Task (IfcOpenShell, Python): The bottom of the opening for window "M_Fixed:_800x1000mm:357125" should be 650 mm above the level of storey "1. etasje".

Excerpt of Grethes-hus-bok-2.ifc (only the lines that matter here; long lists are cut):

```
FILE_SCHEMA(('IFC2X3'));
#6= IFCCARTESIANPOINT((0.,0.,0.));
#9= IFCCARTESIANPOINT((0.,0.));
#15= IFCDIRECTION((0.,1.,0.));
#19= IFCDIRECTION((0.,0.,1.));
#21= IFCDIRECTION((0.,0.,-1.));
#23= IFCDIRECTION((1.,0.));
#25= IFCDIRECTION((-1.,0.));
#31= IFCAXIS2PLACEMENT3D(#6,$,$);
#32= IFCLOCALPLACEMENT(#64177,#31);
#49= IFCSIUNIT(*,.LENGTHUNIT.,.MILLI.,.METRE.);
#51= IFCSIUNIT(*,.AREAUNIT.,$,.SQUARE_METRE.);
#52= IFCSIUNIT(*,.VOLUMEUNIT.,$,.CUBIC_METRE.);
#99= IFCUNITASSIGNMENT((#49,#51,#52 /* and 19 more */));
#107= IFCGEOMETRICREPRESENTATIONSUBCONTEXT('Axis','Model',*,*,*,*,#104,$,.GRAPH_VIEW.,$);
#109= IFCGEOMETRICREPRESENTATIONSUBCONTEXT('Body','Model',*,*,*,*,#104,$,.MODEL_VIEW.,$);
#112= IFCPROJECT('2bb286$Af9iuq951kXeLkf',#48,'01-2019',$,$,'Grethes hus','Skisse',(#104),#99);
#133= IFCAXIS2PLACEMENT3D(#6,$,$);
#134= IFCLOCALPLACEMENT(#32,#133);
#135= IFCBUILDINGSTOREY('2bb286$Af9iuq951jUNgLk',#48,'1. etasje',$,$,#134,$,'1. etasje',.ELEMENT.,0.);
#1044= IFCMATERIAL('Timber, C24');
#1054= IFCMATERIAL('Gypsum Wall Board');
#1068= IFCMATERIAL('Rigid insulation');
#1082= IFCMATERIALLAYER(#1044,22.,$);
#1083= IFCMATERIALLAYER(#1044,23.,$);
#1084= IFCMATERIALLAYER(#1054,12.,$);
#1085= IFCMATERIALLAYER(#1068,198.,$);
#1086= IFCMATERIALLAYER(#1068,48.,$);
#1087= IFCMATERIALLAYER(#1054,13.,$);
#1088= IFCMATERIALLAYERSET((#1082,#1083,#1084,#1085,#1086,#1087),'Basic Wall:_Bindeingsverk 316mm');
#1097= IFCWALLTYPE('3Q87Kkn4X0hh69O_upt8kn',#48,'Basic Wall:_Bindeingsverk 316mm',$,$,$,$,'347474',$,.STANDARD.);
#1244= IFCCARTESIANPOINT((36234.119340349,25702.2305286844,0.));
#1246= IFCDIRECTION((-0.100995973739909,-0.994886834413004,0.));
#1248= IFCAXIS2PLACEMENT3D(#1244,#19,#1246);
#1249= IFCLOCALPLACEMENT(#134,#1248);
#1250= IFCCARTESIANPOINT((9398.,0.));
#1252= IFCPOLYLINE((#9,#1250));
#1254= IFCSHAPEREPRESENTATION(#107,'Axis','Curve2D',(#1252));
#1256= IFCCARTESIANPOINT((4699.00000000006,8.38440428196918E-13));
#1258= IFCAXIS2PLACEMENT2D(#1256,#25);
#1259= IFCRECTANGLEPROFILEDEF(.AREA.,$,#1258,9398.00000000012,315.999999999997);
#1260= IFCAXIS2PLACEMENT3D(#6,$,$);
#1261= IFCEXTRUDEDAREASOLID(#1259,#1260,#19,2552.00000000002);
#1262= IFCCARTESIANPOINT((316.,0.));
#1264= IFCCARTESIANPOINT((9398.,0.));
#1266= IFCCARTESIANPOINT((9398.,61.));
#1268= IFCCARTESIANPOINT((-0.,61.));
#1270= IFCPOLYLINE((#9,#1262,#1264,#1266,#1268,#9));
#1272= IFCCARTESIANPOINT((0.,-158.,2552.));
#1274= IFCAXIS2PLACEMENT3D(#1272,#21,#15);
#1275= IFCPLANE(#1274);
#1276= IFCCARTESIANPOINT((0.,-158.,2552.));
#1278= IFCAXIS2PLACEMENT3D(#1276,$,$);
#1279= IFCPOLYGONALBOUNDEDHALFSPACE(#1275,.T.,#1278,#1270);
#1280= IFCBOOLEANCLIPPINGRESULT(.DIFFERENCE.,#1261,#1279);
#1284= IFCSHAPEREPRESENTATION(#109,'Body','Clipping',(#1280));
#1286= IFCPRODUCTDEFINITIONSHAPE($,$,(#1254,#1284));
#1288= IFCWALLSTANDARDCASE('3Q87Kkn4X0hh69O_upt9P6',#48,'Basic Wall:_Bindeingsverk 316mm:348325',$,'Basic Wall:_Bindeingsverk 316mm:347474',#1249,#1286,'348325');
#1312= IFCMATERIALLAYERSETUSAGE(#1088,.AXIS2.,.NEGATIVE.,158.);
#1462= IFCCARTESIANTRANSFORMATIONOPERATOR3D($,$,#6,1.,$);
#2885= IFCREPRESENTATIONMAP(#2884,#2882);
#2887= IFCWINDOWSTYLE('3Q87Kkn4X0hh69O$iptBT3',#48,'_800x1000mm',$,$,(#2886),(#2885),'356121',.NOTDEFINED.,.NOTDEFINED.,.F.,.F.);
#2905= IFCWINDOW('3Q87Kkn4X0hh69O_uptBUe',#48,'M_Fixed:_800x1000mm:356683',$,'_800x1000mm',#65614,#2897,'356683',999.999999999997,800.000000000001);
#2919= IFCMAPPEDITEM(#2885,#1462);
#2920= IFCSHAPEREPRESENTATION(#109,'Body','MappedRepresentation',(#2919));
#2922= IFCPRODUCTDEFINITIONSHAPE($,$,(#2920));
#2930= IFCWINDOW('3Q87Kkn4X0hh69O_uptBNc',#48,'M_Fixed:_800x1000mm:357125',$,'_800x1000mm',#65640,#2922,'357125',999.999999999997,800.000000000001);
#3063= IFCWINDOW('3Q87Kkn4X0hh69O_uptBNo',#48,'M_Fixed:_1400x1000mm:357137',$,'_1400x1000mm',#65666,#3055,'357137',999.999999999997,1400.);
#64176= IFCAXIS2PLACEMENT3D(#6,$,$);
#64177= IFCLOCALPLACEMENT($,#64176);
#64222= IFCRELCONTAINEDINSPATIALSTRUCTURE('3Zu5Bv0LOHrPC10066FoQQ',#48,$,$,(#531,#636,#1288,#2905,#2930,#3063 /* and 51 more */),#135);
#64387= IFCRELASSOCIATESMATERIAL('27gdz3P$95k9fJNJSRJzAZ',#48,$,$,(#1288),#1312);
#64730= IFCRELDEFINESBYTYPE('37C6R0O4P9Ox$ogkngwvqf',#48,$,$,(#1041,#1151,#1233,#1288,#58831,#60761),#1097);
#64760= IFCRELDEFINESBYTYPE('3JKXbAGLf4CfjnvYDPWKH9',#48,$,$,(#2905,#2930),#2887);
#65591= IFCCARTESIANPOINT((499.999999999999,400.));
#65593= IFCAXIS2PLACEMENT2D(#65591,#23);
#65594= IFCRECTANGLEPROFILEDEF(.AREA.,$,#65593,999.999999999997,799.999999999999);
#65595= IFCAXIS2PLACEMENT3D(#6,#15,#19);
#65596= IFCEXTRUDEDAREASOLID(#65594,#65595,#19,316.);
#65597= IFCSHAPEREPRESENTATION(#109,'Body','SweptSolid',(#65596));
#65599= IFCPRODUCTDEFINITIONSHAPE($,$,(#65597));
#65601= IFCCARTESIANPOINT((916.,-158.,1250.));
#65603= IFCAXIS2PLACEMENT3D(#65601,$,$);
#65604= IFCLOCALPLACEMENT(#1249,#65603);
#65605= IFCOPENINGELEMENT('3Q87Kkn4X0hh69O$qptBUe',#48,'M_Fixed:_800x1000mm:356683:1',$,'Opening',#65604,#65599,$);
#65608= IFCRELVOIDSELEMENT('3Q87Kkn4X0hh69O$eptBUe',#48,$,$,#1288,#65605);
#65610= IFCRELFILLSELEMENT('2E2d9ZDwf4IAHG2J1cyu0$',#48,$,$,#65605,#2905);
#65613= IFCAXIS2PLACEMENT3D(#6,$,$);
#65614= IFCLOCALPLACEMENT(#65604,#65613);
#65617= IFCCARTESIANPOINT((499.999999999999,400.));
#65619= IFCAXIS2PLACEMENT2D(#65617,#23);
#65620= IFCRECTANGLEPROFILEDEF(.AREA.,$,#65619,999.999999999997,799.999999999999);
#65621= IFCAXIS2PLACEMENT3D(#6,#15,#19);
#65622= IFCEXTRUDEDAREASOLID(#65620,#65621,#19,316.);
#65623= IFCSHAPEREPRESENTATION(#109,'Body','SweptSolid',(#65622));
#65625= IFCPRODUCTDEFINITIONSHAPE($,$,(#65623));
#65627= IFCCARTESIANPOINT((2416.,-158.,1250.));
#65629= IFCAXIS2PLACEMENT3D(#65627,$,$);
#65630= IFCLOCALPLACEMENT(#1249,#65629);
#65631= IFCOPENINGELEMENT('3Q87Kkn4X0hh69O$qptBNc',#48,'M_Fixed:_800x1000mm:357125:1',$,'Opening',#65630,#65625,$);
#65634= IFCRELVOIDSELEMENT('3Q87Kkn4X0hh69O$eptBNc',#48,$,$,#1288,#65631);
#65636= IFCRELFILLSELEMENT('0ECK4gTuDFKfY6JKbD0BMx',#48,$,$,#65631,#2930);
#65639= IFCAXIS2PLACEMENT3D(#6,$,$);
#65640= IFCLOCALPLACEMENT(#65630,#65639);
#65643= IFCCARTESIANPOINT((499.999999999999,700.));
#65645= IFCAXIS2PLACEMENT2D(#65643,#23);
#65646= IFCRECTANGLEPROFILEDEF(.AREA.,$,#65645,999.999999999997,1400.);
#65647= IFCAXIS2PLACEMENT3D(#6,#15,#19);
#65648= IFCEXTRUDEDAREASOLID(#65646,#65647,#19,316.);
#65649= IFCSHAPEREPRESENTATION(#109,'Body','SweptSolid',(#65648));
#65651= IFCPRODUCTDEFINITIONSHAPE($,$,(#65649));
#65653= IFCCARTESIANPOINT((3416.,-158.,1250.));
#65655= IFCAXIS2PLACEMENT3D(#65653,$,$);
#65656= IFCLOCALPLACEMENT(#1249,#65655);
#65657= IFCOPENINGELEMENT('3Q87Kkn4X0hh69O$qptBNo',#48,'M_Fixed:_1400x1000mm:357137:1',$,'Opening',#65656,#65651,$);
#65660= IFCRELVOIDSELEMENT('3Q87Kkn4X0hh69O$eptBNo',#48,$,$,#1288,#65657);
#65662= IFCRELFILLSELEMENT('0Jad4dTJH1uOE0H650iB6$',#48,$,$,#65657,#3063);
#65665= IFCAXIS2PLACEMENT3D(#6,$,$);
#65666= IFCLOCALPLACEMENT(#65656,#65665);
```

```python
import numpy as np
import ifcopenshell
import ifcopenshell.api.geometry
import ifcopenshell.geom
import ifcopenshell.util.element
import ifcopenshell.util.placement
import ifcopenshell.util.shape
import ifcopenshell.util.unit

model = ifcopenshell.open("Grethes-hus-bok-2.ifc")
unit_scale = ifcopenshell.util.unit.calculate_unit_scale(model)

window = model.by_guid("3Q87Kkn4X0hh69O_uptBNc")
opening = window.FillsVoids[0].RelatingOpeningElement
storey = ifcopenshell.util.element.get_container(window, ifc_class="IfcBuildingStorey")
level = ifcopenshell.util.placement.get_local_placement(storey.ObjectPlacement)[2, 3]

# The opening's origin need not be at the sill, so measure its lowest point.
shape = ifcopenshell.geom.create_shape(ifcopenshell.geom.settings(), opening)
bottom = ifcopenshell.util.shape.get_shape_bottom_elevation(shape, shape.geometry) / unit_scale
dz = level + 650.0 - bottom

shift = np.array([0.0, 0.0, dz])
# The window is placed relative to its opening, so it follows when the opening moves.
matrix = ifcopenshell.util.placement.get_local_placement(opening.ObjectPlacement)
matrix[:3, 3] += shift
ifcopenshell.api.geometry.edit_object_placement(
    model, product=opening, matrix=matrix, is_si=False, should_transform_children=True
)

print(f"moved by {dz * unit_scale:+.3f} m")

model.write("Grethes-hus-bok-2_updated.ifc")
```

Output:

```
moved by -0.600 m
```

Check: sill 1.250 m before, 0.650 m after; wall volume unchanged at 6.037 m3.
